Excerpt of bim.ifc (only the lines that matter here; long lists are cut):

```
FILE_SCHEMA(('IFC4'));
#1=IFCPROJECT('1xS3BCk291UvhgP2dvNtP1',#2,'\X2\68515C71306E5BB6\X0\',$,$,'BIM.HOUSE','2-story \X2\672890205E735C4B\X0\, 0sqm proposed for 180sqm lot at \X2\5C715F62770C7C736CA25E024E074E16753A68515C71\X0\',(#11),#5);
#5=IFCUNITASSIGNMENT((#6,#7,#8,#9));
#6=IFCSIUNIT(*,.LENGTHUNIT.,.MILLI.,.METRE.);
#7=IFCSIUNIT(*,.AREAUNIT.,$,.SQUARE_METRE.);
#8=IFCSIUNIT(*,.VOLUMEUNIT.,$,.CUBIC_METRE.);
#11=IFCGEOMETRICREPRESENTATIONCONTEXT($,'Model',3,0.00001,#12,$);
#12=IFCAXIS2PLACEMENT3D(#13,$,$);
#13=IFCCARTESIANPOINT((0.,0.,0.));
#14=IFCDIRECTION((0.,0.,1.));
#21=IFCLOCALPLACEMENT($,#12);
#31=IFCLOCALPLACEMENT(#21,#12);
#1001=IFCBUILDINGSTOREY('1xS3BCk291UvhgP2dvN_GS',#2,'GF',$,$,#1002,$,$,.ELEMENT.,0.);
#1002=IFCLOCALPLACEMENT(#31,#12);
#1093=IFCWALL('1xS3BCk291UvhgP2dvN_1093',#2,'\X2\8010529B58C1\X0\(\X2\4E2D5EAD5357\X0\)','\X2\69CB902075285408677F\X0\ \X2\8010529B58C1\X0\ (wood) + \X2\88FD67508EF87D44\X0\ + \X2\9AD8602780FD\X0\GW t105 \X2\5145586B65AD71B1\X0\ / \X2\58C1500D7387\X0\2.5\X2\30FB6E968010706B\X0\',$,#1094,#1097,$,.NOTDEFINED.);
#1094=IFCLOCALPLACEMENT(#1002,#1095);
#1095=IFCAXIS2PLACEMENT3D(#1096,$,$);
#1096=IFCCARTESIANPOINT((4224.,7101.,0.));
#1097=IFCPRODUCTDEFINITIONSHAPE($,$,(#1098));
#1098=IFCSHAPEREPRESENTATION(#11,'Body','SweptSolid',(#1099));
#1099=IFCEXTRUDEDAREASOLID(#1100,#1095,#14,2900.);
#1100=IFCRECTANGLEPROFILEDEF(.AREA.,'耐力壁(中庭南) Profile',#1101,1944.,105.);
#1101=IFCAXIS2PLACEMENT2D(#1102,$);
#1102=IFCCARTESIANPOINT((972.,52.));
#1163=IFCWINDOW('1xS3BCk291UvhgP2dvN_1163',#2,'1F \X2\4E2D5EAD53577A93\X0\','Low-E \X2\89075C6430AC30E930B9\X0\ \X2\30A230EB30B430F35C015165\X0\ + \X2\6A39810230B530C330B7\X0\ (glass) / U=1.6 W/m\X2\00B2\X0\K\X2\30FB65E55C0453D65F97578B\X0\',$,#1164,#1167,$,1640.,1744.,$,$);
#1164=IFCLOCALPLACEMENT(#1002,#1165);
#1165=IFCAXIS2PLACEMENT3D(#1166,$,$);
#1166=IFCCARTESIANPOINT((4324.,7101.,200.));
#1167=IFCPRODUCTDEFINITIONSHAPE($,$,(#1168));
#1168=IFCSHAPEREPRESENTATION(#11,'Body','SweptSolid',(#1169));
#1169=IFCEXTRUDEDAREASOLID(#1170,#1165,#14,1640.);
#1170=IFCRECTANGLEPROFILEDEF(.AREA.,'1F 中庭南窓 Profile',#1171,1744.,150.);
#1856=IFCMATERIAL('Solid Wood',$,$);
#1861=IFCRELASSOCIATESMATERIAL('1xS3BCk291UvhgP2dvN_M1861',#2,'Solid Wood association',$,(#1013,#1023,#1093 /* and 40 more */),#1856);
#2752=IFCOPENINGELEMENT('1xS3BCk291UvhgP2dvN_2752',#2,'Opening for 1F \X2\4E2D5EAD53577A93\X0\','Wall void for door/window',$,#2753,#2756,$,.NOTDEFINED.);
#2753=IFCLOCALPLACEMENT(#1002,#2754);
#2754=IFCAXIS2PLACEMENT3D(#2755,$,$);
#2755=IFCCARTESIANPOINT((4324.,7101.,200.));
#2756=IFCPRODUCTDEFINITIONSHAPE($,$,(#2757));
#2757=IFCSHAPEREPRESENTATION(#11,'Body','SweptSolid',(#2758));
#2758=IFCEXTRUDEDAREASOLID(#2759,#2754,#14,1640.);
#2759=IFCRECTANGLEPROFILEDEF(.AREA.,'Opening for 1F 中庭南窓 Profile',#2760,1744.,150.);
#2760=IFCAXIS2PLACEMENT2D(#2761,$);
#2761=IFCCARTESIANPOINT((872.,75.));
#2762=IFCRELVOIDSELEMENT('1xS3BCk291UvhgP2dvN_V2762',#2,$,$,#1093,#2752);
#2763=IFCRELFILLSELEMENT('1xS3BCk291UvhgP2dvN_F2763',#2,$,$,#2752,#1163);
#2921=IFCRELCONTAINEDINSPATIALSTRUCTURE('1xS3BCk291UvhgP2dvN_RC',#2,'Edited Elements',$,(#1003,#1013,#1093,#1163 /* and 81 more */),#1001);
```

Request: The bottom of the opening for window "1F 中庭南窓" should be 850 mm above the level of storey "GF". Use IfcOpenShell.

```python
import numpy as np
import ifcopenshell
import ifcopenshell.api.geometry
import ifcopenshell.geom
import ifcopenshell.util.element
import ifcopenshell.util.placement
import ifcopenshell.util.shape
import ifcopenshell.util.unit

model = ifcopenshell.open("bim.ifc")
unit_scale = ifcopenshell.util.unit.calculate_unit_scale(model)

window = model.by_guid("1xS3BCk291UvhgP2dvN_1163")
opening = window.FillsVoids[0].RelatingOpeningElement
storey = ifcopenshell.util.element.get_container(window, ifc_class="IfcBuildingStorey")
level = ifcopenshell.util.placement.get_local_placement(storey.ObjectPlacement)[2, 3]

# The opening's origin need not be at the sill, so measure its lowest point.
shape = ifcopenshell.geom.create_shape(ifcopenshell.geom.settings(), opening)
bottom = ifcopenshell.util.shape.get_shape_bottom_elevation(shape, shape.geometry) / unit_scale
dz = level + 850.0 - bottom

shift = np.array([0.0, 0.0, dz])
# The window is not placed relative to its opening, so move both.
for product in (opening, window):
    matrix = ifcopenshell.util.placement.get_local_placement(product.ObjectPlacement)
    matrix[:3, 3] += shift
    ifcopenshell.api.geometry.edit_object_placement(model, product=product, matrix=matrix, is_si=False)

print(f"moved by {dz * unit_scale:+.3f} m")

model.write("bim_rev.ifc")
```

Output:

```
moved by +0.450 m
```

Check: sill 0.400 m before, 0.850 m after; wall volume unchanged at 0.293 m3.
